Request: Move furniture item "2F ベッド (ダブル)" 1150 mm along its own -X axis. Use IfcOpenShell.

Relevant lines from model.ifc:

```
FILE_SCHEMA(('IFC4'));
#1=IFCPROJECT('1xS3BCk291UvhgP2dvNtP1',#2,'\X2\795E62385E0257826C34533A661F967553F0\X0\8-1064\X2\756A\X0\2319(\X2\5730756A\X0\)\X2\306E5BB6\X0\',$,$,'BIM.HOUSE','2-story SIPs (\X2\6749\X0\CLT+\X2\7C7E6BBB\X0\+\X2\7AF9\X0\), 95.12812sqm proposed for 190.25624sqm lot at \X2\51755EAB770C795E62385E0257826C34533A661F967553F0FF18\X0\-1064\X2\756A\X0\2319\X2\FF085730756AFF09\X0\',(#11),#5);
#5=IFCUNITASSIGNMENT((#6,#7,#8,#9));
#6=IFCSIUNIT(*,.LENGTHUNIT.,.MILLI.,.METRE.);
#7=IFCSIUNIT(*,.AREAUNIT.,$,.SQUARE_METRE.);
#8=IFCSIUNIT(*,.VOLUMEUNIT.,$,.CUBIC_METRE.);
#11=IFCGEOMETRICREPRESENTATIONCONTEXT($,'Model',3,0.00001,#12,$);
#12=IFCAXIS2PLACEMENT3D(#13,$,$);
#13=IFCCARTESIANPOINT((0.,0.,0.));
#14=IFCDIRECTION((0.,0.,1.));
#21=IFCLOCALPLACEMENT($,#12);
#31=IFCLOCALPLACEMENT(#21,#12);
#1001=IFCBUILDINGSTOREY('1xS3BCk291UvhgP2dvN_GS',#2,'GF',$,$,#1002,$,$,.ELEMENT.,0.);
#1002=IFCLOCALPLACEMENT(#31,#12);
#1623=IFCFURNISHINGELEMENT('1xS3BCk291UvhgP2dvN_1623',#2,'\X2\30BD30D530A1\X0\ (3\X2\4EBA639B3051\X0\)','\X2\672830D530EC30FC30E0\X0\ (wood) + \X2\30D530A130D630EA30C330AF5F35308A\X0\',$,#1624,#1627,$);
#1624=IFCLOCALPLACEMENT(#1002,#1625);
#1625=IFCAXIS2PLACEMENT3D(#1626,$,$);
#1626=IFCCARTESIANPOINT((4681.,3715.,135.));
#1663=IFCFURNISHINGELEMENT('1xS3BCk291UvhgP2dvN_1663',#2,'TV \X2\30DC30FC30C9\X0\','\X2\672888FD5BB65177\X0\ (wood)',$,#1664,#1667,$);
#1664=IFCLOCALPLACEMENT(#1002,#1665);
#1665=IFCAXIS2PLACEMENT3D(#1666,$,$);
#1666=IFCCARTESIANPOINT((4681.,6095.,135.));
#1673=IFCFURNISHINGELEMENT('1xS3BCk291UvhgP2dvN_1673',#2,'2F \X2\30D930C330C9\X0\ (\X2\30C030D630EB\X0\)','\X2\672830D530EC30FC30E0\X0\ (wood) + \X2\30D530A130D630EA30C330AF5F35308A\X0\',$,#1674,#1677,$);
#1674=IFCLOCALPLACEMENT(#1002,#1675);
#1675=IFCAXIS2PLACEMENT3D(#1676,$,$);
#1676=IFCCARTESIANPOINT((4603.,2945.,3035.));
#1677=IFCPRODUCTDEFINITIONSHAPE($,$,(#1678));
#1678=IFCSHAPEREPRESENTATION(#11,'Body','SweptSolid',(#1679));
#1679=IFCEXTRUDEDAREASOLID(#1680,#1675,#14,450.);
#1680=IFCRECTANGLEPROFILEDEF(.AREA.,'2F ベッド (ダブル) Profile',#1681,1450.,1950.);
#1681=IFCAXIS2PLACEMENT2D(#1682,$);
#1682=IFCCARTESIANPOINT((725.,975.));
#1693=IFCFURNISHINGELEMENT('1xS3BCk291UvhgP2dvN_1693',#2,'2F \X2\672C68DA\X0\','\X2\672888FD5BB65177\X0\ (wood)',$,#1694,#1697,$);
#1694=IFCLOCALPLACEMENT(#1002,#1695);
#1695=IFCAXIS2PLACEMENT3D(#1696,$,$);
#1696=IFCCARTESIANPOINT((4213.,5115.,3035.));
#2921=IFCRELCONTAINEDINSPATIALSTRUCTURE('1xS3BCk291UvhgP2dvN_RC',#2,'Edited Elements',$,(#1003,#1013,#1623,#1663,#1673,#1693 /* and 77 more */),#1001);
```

```python
import ifcopenshell
import ifcopenshell.api.geometry
import ifcopenshell.util.placement
import ifcopenshell.util.unit

model = ifcopenshell.open("model.ifc")
unit_scale = ifcopenshell.util.unit.calculate_unit_scale(model)

item = model.by_guid("1xS3BCk291UvhgP2dvN_1673")
matrix = ifcopenshell.util.placement.get_local_placement(item.ObjectPlacement)
matrix[:3, 3] -= matrix[:3, 0] * 1.15 / unit_scale
ifcopenshell.api.geometry.edit_object_placement(model, product=item, matrix=matrix, is_si=False)

print(ifcopenshell.util.placement.get_local_placement(item.ObjectPlacement).round(3) + 0.0)

model.write("model-out.ifc")
```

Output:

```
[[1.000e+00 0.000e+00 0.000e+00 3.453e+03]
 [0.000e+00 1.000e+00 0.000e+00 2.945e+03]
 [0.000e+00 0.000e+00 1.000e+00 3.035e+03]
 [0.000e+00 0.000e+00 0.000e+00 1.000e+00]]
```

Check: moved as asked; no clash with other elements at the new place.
